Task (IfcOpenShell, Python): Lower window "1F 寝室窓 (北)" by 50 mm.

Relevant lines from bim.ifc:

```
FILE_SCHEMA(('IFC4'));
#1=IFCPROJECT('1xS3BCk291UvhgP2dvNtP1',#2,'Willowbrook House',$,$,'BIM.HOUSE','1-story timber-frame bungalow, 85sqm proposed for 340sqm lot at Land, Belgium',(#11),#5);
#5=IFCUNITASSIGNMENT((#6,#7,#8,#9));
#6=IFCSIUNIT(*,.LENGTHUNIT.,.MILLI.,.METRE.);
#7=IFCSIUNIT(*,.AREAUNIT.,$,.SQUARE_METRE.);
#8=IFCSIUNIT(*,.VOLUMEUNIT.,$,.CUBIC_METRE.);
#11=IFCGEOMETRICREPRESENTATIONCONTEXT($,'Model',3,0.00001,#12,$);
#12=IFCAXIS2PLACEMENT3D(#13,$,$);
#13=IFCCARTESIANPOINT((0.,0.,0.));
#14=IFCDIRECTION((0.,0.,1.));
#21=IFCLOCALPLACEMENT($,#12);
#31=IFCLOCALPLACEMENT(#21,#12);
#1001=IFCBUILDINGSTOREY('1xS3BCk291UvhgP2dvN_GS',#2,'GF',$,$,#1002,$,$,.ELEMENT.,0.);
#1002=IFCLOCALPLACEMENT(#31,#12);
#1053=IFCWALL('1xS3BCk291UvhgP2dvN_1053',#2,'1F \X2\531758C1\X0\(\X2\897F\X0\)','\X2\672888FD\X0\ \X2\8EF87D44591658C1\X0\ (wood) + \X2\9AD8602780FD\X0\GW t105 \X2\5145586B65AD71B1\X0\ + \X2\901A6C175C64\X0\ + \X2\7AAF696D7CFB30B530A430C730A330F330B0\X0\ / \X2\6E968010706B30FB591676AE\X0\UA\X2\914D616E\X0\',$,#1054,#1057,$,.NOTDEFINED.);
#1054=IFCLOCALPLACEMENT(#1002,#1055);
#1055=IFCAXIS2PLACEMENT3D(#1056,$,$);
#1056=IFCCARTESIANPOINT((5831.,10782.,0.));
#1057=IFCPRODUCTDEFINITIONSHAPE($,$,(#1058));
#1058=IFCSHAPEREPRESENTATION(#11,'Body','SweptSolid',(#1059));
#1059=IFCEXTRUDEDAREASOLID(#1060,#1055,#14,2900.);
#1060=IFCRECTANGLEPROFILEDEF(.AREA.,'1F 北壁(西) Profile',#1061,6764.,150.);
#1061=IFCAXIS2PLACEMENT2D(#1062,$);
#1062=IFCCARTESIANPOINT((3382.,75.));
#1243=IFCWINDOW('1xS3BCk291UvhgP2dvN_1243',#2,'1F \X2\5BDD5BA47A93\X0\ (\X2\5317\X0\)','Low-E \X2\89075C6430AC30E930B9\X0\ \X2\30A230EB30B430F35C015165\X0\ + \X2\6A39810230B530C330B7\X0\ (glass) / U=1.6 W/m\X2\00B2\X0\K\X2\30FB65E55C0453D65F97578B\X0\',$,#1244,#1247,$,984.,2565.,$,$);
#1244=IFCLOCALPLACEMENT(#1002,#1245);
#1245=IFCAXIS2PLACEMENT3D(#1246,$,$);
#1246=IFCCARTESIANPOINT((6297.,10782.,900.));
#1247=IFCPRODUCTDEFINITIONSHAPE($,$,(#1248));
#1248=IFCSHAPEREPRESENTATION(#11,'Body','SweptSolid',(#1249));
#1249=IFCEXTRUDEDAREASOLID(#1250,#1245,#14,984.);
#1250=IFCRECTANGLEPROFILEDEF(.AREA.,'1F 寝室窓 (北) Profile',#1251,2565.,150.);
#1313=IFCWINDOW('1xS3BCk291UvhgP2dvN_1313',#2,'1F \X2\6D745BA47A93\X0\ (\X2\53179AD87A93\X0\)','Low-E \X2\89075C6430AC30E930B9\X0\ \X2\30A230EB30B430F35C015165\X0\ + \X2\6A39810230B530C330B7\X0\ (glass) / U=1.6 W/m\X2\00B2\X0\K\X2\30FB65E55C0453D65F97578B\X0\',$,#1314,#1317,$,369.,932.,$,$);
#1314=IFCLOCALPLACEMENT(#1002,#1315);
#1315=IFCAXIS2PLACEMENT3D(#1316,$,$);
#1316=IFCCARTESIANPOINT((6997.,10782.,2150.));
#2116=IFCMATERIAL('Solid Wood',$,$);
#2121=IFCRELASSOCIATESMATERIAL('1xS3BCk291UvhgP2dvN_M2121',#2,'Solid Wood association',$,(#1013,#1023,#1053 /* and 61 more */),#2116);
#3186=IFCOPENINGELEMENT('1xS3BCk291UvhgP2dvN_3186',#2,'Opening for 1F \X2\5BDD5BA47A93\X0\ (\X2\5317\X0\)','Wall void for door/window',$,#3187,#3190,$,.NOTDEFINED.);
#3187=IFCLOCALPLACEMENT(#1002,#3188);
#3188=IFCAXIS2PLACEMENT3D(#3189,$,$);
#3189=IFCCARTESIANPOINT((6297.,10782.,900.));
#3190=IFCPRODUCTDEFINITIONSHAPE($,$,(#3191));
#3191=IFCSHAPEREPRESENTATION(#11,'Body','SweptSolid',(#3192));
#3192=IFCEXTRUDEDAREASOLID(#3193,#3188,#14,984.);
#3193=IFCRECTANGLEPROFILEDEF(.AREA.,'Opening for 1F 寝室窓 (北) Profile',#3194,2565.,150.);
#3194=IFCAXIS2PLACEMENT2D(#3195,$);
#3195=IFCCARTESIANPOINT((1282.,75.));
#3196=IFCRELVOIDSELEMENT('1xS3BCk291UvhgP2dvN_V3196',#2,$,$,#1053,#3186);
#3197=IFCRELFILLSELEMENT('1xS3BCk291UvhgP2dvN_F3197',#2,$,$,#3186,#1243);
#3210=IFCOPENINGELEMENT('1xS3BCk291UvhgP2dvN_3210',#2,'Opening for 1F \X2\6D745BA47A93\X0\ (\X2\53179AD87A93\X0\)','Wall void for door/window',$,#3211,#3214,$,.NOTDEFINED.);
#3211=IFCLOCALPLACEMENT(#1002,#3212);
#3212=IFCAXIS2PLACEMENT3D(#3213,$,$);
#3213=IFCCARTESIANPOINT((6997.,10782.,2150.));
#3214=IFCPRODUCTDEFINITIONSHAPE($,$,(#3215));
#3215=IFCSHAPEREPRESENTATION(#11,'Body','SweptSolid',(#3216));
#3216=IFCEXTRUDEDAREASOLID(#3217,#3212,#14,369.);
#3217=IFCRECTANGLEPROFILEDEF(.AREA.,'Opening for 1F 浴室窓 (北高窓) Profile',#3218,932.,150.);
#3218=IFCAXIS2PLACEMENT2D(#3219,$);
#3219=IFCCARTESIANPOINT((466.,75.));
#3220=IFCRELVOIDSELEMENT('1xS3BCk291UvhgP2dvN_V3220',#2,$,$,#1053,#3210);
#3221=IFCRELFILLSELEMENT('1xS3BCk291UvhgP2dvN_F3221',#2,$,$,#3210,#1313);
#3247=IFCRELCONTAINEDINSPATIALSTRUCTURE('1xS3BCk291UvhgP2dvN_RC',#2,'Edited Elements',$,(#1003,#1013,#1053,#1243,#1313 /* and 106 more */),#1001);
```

```python
import numpy as np
import ifcopenshell
import ifcopenshell.api.geometry
import ifcopenshell.util.placement
import ifcopenshell.util.unit

model = ifcopenshell.open("bim.ifc")
unit_scale = ifcopenshell.util.unit.calculate_unit_scale(model)

window = model.by_guid("1xS3BCk291UvhgP2dvN_1243")
opening = window.FillsVoids[0].RelatingOpeningElement
dz = -0.05 / unit_scale

shift = np.array([0.0, 0.0, dz])
# The window is not placed relative to its opening, so move both.
for product in (opening, window):
    matrix = ifcopenshell.util.placement.get_local_placement(product.ObjectPlacement)
    matrix[:3, 3] += shift
    ifcopenshell.api.geometry.edit_object_placement(model, product=product, matrix=matrix, is_si=False)

print(f"moved by {dz * unit_scale:+.3f} m")

model.write("bim_rev.ifc")
```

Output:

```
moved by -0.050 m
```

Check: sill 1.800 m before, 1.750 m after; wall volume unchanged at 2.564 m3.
